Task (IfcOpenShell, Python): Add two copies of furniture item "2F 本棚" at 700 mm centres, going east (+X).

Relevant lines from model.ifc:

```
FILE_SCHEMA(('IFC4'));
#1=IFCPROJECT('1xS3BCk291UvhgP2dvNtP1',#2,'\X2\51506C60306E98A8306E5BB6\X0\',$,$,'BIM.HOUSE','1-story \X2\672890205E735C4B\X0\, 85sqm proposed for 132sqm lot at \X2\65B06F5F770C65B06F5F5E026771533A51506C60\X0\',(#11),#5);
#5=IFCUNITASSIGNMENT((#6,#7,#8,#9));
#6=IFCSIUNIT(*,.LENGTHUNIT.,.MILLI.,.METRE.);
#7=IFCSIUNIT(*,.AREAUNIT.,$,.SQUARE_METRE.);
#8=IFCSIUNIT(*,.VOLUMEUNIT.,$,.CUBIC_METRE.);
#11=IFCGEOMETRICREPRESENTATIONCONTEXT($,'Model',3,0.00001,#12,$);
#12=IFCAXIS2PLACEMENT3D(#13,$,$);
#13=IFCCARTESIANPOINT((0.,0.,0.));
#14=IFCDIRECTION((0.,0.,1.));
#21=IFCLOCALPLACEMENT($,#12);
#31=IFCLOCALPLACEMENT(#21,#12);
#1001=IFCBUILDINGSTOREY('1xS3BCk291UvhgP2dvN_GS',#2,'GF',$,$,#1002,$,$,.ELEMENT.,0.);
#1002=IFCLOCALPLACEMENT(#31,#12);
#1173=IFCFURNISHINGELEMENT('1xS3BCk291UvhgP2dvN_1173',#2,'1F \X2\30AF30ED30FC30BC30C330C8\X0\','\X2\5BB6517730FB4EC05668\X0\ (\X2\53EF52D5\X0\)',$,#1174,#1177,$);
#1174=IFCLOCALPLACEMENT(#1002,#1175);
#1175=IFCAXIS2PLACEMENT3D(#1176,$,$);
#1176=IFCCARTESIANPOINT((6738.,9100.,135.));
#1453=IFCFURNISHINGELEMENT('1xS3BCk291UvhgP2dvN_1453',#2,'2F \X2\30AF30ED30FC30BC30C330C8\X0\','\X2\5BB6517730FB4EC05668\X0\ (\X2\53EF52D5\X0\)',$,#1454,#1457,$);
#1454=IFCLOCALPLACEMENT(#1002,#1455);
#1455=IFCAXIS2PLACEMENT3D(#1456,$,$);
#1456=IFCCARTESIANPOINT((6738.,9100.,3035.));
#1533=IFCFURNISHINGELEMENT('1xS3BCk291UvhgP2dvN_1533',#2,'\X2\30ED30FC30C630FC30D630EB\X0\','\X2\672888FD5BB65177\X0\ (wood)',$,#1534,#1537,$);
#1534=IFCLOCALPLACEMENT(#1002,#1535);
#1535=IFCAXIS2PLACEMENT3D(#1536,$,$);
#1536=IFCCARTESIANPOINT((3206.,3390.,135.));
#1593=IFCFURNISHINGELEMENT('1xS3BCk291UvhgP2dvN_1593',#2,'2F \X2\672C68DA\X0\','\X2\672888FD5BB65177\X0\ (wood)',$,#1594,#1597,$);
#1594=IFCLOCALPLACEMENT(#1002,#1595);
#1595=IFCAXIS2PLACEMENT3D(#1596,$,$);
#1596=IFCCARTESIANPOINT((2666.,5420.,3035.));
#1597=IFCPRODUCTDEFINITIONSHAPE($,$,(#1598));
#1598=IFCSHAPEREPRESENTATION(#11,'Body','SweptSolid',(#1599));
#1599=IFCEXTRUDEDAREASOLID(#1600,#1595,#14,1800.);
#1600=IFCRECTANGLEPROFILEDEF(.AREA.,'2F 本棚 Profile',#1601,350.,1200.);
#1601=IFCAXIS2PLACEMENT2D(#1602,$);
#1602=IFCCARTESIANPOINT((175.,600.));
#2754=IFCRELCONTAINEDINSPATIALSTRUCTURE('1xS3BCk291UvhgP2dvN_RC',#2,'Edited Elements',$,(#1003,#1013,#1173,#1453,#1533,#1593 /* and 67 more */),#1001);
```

```python
import numpy as np
import ifcopenshell
import ifcopenshell.api.geometry
import ifcopenshell.api.root
import ifcopenshell.util.element
import ifcopenshell.util.placement

model = ifcopenshell.open("model.ifc")


def reuse_history(source, copy):
    """copy_class also copies each property set's owner history, people and application; keep the originals."""
    for rel in copy.IsDefinedBy:
        if rel.is_a("IfcRelDefinesByProperties") and (history := rel.RelatingPropertyDefinition.OwnerHistory):
            rel.RelatingPropertyDefinition.OwnerHistory = source.OwnerHistory
            ifcopenshell.util.element.remove_deep2(model, history)


source = model.by_guid("1xS3BCk291UvhgP2dvN_1593")
base = ifcopenshell.util.placement.get_local_placement(source.ObjectPlacement)
step = np.array([1.0, 0.0, 0.0]) * 700.0

for i in range(1, 3):
    copy = ifcopenshell.api.root.copy_class(model, product=source)
    copy.Representation = ifcopenshell.util.element.copy_deep(
        model, source.Representation, exclude=["IfcGeometricRepresentationContext", "IfcRepresentationMap"]
    )
    reuse_history(source, copy)
    matrix = base.copy()
    matrix[:3, 3] += i * step
    print("added at", matrix[:3, 3].round(3) + 0.0)
    ifcopenshell.api.geometry.edit_object_placement(model, product=copy, matrix=matrix, is_si=False)

model.write("model_v2.ifc")
```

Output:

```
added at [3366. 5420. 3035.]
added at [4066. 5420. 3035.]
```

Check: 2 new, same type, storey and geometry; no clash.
